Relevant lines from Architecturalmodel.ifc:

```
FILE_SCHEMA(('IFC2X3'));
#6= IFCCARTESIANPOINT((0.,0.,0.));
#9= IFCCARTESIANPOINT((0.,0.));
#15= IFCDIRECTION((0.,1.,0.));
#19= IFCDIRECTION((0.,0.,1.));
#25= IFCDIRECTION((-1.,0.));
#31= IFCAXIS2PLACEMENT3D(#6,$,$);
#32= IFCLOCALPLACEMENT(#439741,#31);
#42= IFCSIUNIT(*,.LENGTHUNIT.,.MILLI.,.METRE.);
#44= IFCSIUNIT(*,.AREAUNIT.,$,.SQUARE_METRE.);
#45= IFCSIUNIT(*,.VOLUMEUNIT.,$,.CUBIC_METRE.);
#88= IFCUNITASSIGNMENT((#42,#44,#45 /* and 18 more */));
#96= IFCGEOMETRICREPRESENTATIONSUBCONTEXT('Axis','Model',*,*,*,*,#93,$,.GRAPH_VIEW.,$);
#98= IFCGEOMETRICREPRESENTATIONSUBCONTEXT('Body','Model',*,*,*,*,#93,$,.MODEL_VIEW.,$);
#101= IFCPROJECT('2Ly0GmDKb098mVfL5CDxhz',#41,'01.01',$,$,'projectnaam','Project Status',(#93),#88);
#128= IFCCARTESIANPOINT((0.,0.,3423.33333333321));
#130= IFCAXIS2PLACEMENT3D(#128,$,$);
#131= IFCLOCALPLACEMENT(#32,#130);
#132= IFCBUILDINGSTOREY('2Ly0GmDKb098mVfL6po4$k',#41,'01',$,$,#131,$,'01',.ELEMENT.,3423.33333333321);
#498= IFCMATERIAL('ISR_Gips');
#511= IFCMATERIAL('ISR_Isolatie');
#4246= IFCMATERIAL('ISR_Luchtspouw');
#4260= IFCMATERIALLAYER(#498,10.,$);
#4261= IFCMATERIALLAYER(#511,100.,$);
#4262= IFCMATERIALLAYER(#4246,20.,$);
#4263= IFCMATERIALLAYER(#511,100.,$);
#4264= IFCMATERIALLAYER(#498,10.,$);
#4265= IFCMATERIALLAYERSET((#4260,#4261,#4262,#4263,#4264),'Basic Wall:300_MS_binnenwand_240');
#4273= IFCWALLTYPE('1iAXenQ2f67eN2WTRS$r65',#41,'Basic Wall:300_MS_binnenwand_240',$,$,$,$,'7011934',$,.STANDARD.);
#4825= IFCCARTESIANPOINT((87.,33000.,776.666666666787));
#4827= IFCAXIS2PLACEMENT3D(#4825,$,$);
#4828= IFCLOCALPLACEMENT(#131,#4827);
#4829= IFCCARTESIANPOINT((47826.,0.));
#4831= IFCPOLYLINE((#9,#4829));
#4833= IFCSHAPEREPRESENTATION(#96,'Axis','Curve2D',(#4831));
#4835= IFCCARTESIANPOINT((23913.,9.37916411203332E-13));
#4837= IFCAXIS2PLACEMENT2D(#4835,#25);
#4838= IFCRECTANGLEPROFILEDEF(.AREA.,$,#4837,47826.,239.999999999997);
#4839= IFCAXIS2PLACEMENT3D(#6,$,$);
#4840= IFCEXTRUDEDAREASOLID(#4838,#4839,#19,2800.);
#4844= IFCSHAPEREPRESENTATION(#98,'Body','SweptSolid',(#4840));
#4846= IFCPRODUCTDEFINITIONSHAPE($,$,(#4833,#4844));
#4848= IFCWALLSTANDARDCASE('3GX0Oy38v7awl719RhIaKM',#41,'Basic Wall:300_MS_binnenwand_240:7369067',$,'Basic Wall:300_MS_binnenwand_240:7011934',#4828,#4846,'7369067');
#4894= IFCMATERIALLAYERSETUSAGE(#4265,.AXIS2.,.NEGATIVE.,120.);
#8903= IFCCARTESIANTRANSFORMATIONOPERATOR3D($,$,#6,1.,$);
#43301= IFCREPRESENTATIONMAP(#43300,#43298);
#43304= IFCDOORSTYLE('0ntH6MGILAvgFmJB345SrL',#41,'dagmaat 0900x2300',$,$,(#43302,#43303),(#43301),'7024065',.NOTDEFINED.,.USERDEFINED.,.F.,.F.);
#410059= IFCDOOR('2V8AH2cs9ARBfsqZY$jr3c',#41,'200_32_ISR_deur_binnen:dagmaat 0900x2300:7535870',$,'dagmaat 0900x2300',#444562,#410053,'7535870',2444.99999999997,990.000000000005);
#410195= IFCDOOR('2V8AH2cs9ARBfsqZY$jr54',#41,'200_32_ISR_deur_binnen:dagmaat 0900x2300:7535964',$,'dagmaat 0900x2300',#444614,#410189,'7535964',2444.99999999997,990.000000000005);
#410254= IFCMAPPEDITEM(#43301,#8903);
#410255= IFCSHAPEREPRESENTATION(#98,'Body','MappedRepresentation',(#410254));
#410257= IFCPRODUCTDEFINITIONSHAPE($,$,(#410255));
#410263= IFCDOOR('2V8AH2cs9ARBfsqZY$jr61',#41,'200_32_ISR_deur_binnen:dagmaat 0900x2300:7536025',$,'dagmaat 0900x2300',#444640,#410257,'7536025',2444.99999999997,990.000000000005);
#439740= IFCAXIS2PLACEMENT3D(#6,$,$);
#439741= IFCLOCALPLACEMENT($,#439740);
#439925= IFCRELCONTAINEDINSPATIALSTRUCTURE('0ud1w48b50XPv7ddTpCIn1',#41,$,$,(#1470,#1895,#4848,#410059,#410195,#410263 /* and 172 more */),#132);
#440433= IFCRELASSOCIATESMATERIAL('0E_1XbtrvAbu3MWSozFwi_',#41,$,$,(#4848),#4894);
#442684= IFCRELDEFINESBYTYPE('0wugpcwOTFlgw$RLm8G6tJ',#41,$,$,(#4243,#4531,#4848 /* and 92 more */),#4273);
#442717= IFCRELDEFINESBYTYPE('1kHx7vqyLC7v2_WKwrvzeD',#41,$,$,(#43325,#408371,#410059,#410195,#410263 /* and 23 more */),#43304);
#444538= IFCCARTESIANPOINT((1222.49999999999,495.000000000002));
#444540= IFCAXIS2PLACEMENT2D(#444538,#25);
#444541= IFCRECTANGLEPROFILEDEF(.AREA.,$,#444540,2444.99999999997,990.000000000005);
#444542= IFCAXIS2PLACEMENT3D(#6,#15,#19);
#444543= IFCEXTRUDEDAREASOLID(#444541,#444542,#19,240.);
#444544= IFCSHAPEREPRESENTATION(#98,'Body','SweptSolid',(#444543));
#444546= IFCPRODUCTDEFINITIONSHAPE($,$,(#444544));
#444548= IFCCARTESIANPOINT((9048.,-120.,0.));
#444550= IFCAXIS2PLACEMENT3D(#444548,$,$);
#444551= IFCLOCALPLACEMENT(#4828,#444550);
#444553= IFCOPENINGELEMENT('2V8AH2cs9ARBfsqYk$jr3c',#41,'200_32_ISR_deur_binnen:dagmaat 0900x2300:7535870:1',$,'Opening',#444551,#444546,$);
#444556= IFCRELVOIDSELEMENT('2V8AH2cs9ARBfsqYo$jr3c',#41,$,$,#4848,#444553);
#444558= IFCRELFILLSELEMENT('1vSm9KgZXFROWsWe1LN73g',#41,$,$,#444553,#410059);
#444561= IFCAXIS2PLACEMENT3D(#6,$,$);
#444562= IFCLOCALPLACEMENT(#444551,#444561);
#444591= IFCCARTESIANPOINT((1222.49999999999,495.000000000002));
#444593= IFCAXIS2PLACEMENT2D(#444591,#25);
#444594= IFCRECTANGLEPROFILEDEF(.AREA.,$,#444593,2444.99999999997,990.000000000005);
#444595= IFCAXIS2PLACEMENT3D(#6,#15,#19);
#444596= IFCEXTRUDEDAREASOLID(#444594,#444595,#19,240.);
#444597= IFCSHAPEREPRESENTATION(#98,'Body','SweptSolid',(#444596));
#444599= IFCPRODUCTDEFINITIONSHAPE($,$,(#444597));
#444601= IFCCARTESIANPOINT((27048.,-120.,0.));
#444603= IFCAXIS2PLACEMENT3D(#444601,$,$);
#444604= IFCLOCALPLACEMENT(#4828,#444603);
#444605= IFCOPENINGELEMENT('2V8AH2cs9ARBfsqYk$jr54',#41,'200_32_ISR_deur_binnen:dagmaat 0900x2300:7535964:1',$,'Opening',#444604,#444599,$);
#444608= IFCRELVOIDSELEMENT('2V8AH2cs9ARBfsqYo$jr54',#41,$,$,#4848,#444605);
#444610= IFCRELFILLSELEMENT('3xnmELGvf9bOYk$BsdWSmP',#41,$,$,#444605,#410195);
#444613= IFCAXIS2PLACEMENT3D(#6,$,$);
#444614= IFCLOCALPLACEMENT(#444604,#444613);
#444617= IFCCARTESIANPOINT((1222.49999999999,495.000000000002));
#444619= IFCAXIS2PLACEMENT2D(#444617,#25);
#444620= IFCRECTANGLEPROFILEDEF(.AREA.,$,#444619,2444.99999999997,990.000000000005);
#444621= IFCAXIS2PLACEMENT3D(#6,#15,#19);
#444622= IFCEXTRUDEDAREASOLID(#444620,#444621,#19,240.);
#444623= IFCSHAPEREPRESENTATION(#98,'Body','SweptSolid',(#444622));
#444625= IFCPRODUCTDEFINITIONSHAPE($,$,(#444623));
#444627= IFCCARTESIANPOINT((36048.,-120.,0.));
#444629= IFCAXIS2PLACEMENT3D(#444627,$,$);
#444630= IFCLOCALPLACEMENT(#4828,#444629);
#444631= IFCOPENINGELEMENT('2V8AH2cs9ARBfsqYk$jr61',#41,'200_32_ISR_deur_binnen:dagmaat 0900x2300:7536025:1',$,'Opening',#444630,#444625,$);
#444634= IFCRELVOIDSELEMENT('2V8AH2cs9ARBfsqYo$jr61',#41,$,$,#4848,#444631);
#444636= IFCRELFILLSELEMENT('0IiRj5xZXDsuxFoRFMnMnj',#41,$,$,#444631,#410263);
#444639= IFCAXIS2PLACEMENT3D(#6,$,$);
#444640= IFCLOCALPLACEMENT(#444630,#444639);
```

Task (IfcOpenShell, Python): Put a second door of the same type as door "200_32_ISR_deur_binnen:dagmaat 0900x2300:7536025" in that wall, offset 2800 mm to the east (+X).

```python
import ifcopenshell
import ifcopenshell.api.feature
import ifcopenshell.api.geometry
import ifcopenshell.api.root
import ifcopenshell.geom
import ifcopenshell.util.element
import ifcopenshell.util.placement
import ifcopenshell.util.shape
import ifcopenshell.util.unit

model = ifcopenshell.open("Architecturalmodel.ifc")
unit_scale = ifcopenshell.util.unit.calculate_unit_scale(model)
settings = ifcopenshell.geom.settings()


def volume(element):
    """Net volume in cubic metres, openings subtracted."""
    shape = ifcopenshell.geom.create_shape(settings, element)
    return ifcopenshell.util.shape.get_volume(shape.geometry)


def reuse_history(source, copy):
    """copy_class also copies each property set's owner history, people and application; keep the originals."""
    for rel in copy.IsDefinedBy:
        if rel.is_a("IfcRelDefinesByProperties") and (history := rel.RelatingPropertyDefinition.OwnerHistory):
            rel.RelatingPropertyDefinition.OwnerHistory = source.OwnerHistory
            ifcopenshell.util.element.remove_deep2(model, history)


door = model.by_id(410263)
opening = door.FillsVoids[0].RelatingOpeningElement
wall = opening.VoidsElements[0].RelatingBuildingElement
before = volume(wall)
shift = ifcopenshell.util.placement.get_local_placement(wall.ObjectPlacement)[:3, 0] * 2.8 / unit_scale

# copy_class copies the void relationship, type, container and properties, but no geometry.
new_opening = ifcopenshell.api.root.copy_class(model, product=opening)
new_opening.Representation = ifcopenshell.util.element.copy_deep(
    model, opening.Representation, exclude=["IfcGeometricRepresentationContext", "IfcRepresentationMap"]
)
new_opening.Name = "200_32_ISR_deur_binnen:dagmaat 0900x2300"
new_door = ifcopenshell.api.root.copy_class(model, product=door)
new_door.Representation = ifcopenshell.util.element.copy_deep(
    model, door.Representation, exclude=["IfcGeometricRepresentationContext", "IfcRepresentationMap"]
)
new_door.Name = "200_32_ISR_deur_binnen:dagmaat 0900x2300"
new_door.Tag = None
reuse_history(door, new_door)
fills = ifcopenshell.api.feature.add_filling(model, opening=new_opening, element=new_door)
fills.OwnerHistory = new_door.OwnerHistory  # required in IFC2X3

for old, new in ((opening, new_opening), (door, new_door)):
    matrix = ifcopenshell.util.placement.get_local_placement(old.ObjectPlacement)
    matrix[:3, 3] += shift
    ifcopenshell.api.geometry.edit_object_placement(model, product=new, matrix=matrix, is_si=False)

after = volume(wall)

print(f"wall volume {before:.3f} -> {after:.3f} m3")

model.write("Architecturalmodel_rev.ifc")
```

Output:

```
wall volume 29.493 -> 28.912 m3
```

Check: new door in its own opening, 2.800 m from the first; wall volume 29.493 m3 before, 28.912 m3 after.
